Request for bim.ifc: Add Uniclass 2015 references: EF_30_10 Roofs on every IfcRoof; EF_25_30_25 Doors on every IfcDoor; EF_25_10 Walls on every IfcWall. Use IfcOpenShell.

First a look at what the model holds.

```python
import ifcopenshell

model = ifcopenshell.open("bim.ifc")
print(model.schema)
print("classifications:", [c.Name for c in model.by_type("IfcClassification")])
for ifc_class in ("IfcDoor", "IfcRoof", "IfcStair", "IfcWall", "IfcWindow"):
    print(ifc_class, len(model.by_type(ifc_class)))
```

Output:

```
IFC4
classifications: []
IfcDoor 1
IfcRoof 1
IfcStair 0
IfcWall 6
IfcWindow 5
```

```python
import ifcopenshell
import ifcopenshell.api.classification

model = ifcopenshell.open("bim.ifc")

system = ifcopenshell.api.classification.add_classification(model, classification="Uniclass 2015")

codes = {
    "IfcRoof": ("EF_30_10", "Roofs"),
    "IfcDoor": ("EF_25_30_25", "Doors"),
    "IfcWall": ("EF_25_10", "Walls"),
}
for ifc_class, (code, name) in codes.items():
    products = model.by_type(ifc_class)
    ifcopenshell.api.classification.add_reference(
        model, products=products, classification=system, identification=code, name=name
    )
    print(code, len(products))

model.write("bim_rev.ifc")
```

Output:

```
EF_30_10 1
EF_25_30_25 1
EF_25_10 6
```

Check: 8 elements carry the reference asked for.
